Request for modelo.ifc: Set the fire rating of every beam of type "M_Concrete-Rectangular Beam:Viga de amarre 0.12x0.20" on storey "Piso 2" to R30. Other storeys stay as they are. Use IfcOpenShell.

First a look at what the model holds.

```python
import ifcopenshell
import ifcopenshell.util.element

model = ifcopenshell.open("modelo.ifc")
print(model.schema)
storey = next(s for s in model.by_type("IfcBuildingStorey") if s.Name == "Piso 2")
beams = [e for e in ifcopenshell.util.element.get_decomposition(storey) if e.is_a("IfcBeam")]
seen = {}
for e in beams:
    element_type = ifcopenshell.util.element.get_type(e)
    key = (element_type.Name if element_type != e and element_type else None, ifcopenshell.util.element.get_pset(e, "Pset_BeamCommon", "FireRating"))
    seen[key] = seen.get(key, 0) + 1
for (name, value), count in sorted(seen.items(), key=str):
    print(count, "x", name, "|", value)
```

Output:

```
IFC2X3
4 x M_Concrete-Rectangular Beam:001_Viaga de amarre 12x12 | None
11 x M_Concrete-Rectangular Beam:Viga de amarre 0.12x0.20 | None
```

```python
import ifcopenshell
import ifcopenshell.api.pset
import ifcopenshell.util.element

model = ifcopenshell.open("modelo.ifc")

storey = next(s for s in model.by_type("IfcBuildingStorey") if s.Name == "Piso 2")
beams = [e for e in ifcopenshell.util.element.get_decomposition(storey) if e.is_a("IfcBeam")]

count = 0
for e in beams:
    element_type = ifcopenshell.util.element.get_type(e)
    if element_type in (None, e) or element_type.Name != "M_Concrete-Rectangular Beam:Viga de amarre 0.12x0.20":
        continue
    # add_pset returns the element's existing set when there is one.
    pset = ifcopenshell.api.pset.add_pset(model, product=e, name="Pset_BeamCommon")
    ifcopenshell.api.pset.edit_pset(model, pset=pset, properties={"FireRating": "R30"})
    count += 1

print(count, "beams updated")

model.write("modelo_rev.ifc")
```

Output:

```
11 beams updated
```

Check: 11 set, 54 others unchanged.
